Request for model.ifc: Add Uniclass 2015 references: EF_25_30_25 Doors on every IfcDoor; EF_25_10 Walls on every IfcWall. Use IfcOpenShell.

First a look at what the model holds.

```python
import ifcopenshell

model = ifcopenshell.open("model.ifc")
print(model.schema)
print("classifications:", [c.Name for c in model.by_type("IfcClassification")])
for ifc_class in ("IfcDoor", "IfcRoof", "IfcStair", "IfcWall", "IfcWindow"):
    print(ifc_class, len(model.by_type(ifc_class)))
```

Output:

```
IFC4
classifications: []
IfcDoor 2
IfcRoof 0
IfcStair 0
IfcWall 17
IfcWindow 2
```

```python
import ifcopenshell
import ifcopenshell.api.classification

model = ifcopenshell.open("model.ifc")

system = ifcopenshell.api.classification.add_classification(model, classification="Uniclass 2015")

codes = {
    "IfcDoor": ("EF_25_30_25", "Doors"),
    "IfcWall": ("EF_25_10", "Walls"),
}
for ifc_class, (code, name) in codes.items():
    products = model.by_type(ifc_class)
    ifcopenshell.api.classification.add_reference(
        model, products=products, classification=system, identification=code, name=name
    )
    print(code, len(products))

model.write("model-out.ifc")
```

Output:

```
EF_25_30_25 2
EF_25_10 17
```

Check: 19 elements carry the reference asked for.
